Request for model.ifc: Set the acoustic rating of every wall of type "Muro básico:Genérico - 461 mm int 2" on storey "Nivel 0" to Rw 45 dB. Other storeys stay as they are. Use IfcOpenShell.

First a look at what the model holds.

```python
import ifcopenshell
import ifcopenshell.util.element

model = ifcopenshell.open("model.ifc")
print(model.schema)
storey = next(s for s in model.by_type("IfcBuildingStorey") if s.Name == "Nivel 0")
walls = [e for e in ifcopenshell.util.element.get_decomposition(storey) if e.is_a("IfcWall")]
seen = {}
for e in walls:
    element_type = ifcopenshell.util.element.get_type(e)
    key = (element_type.Name if element_type != e and element_type else None, ifcopenshell.util.element.get_pset(e, "Pset_WallCommon", "AcousticRating"))
    seen[key] = seen.get(key, 0) + 1
for (name, value), count in sorted(seen.items(), key=str):
    print(count, "x", name, "|", value)
```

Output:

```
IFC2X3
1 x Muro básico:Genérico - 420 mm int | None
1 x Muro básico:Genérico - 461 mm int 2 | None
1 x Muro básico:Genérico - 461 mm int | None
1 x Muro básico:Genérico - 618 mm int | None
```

```python
import ifcopenshell
import ifcopenshell.api.pset
import ifcopenshell.util.element

model = ifcopenshell.open("model.ifc")

storey = next(s for s in model.by_type("IfcBuildingStorey") if s.Name == "Nivel 0")
walls = [e for e in ifcopenshell.util.element.get_decomposition(storey) if e.is_a("IfcWall")]

count = 0
for e in walls:
    element_type = ifcopenshell.util.element.get_type(e)
    if element_type in (None, e) or element_type.Name != "Muro básico:Genérico - 461 mm int 2":
        continue
    # add_pset returns the element's existing set when there is one.
    pset = ifcopenshell.api.pset.add_pset(model, product=e, name="Pset_WallCommon")
    ifcopenshell.api.pset.edit_pset(model, pset=pset, properties={"AcousticRating": "Rw 45 dB"})
    count += 1

print(count, "walls updated")

model.write("model_rev.ifc")
```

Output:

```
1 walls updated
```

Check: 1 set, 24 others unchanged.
